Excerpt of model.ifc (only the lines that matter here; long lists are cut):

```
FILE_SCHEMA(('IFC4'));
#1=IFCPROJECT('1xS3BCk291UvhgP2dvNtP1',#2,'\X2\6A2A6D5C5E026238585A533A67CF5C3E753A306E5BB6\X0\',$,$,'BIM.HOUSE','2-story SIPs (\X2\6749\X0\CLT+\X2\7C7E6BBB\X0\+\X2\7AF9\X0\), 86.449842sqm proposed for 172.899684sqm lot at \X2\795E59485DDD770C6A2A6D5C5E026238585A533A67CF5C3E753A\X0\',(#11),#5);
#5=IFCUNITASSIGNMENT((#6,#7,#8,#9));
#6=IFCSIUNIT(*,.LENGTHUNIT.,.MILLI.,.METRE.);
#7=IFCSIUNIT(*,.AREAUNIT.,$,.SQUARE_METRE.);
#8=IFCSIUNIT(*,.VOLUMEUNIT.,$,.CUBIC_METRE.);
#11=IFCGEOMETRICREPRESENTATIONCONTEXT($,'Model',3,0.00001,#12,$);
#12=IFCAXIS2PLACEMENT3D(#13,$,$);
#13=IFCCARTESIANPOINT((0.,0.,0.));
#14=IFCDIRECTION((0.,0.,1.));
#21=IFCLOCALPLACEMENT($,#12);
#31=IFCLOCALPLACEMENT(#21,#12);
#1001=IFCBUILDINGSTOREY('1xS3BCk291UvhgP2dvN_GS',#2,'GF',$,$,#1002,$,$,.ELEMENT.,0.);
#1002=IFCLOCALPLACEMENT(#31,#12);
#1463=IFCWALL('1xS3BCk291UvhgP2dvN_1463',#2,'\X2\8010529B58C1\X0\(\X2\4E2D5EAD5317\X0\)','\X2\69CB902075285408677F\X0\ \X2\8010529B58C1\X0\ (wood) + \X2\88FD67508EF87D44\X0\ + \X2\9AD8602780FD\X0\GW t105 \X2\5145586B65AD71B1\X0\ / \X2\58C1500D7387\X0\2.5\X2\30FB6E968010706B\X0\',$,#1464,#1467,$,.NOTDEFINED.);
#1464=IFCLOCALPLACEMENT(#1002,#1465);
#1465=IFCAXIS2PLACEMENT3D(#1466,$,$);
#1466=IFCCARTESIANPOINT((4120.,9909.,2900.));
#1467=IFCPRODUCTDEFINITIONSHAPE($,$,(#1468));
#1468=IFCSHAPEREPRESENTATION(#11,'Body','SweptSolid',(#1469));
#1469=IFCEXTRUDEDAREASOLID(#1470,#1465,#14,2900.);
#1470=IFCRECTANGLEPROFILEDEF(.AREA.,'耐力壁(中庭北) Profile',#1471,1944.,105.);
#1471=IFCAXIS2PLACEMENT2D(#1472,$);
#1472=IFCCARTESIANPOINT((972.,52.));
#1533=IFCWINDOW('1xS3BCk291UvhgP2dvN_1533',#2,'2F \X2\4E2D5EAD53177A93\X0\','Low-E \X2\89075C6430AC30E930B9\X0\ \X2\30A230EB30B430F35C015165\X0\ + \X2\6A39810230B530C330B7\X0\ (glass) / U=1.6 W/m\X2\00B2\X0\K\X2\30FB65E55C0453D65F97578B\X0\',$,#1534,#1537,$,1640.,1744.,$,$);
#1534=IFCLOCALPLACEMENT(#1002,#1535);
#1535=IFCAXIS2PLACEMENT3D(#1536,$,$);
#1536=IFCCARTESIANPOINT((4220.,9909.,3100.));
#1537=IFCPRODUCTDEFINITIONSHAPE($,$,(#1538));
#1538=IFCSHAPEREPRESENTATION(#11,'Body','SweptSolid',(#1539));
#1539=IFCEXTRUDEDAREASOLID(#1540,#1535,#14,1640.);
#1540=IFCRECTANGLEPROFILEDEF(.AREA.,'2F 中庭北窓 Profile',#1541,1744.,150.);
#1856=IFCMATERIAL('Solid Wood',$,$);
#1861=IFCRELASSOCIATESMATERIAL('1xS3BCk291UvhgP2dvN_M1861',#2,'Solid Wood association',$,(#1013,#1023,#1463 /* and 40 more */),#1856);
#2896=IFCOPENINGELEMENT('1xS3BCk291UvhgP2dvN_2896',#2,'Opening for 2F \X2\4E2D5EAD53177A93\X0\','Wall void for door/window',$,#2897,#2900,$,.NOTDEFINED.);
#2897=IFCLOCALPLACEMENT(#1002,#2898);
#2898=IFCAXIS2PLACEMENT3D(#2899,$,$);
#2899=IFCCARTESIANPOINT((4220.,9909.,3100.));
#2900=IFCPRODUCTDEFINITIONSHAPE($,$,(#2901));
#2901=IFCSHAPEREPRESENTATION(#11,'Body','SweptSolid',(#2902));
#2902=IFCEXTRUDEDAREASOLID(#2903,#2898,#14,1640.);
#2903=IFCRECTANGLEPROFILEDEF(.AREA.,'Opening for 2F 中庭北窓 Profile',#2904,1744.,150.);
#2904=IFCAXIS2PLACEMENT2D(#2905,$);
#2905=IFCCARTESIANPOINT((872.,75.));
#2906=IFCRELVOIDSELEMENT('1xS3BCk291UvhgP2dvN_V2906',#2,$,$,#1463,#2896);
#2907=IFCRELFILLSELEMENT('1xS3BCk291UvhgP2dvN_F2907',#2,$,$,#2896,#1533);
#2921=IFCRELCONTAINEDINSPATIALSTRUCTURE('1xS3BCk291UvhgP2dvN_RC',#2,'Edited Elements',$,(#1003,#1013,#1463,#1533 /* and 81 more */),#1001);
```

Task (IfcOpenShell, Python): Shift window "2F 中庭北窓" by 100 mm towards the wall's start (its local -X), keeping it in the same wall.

```python
import ifcopenshell
import ifcopenshell.api.geometry
import ifcopenshell.util.placement
import ifcopenshell.util.unit

model = ifcopenshell.open("model.ifc")
unit_scale = ifcopenshell.util.unit.calculate_unit_scale(model)

window = model.by_guid("1xS3BCk291UvhgP2dvN_1533")
opening = window.FillsVoids[0].RelatingOpeningElement
wall = opening.VoidsElements[0].RelatingBuildingElement

wall_matrix = ifcopenshell.util.placement.get_local_placement(wall.ObjectPlacement)
shift = wall_matrix[:3, 0] * -0.1 / unit_scale
before = ifcopenshell.util.placement.get_local_placement(window.ObjectPlacement)[:3, 3].copy()

# The window is not placed relative to its opening, so move both.
for product in (opening, window):
    matrix = ifcopenshell.util.placement.get_local_placement(product.ObjectPlacement)
    matrix[:3, 3] += shift
    ifcopenshell.api.geometry.edit_object_placement(model, product=product, matrix=matrix, is_si=False)

after = ifcopenshell.util.placement.get_local_placement(window.ObjectPlacement)[:3, 3]
print("window moved by", (after - before).round(3) + 0.0)

model.write("model_edited.ifc")
```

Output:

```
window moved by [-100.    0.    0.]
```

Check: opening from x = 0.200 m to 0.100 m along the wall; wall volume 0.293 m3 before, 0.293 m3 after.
